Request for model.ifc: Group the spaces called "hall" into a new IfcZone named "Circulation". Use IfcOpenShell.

First a look at what the model holds.

```python
import ifcopenshell

model = ifcopenshell.open("model.ifc")
print(model.schema)
seen = {}
for space in model.by_type("IfcSpace"):
    seen[space.LongName] = seen.get(space.LongName, 0) + 1
for name, count in sorted(seen.items(), key=str):
    print(count, "x", name)
print("zones:", [z.Name for z in model.by_type("IfcZone")][:20])
```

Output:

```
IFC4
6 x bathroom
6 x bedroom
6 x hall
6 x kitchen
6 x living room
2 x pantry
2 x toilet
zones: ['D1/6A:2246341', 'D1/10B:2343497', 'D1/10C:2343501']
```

```python
import ifcopenshell
import ifcopenshell.api.group
import ifcopenshell.api.root

model = ifcopenshell.open("model.ifc")

names = {"hall"}
spaces = [s for s in model.by_type("IfcSpace") if s.LongName in names]

zone = ifcopenshell.api.root.create_entity(model, ifc_class="IfcZone", name="Circulation")
ifcopenshell.api.group.assign_group(model, products=spaces, group=zone)
print(len(spaces), "spaces in", zone.Name)

model.write("model_rev.ifc")
```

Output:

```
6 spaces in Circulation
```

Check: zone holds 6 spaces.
